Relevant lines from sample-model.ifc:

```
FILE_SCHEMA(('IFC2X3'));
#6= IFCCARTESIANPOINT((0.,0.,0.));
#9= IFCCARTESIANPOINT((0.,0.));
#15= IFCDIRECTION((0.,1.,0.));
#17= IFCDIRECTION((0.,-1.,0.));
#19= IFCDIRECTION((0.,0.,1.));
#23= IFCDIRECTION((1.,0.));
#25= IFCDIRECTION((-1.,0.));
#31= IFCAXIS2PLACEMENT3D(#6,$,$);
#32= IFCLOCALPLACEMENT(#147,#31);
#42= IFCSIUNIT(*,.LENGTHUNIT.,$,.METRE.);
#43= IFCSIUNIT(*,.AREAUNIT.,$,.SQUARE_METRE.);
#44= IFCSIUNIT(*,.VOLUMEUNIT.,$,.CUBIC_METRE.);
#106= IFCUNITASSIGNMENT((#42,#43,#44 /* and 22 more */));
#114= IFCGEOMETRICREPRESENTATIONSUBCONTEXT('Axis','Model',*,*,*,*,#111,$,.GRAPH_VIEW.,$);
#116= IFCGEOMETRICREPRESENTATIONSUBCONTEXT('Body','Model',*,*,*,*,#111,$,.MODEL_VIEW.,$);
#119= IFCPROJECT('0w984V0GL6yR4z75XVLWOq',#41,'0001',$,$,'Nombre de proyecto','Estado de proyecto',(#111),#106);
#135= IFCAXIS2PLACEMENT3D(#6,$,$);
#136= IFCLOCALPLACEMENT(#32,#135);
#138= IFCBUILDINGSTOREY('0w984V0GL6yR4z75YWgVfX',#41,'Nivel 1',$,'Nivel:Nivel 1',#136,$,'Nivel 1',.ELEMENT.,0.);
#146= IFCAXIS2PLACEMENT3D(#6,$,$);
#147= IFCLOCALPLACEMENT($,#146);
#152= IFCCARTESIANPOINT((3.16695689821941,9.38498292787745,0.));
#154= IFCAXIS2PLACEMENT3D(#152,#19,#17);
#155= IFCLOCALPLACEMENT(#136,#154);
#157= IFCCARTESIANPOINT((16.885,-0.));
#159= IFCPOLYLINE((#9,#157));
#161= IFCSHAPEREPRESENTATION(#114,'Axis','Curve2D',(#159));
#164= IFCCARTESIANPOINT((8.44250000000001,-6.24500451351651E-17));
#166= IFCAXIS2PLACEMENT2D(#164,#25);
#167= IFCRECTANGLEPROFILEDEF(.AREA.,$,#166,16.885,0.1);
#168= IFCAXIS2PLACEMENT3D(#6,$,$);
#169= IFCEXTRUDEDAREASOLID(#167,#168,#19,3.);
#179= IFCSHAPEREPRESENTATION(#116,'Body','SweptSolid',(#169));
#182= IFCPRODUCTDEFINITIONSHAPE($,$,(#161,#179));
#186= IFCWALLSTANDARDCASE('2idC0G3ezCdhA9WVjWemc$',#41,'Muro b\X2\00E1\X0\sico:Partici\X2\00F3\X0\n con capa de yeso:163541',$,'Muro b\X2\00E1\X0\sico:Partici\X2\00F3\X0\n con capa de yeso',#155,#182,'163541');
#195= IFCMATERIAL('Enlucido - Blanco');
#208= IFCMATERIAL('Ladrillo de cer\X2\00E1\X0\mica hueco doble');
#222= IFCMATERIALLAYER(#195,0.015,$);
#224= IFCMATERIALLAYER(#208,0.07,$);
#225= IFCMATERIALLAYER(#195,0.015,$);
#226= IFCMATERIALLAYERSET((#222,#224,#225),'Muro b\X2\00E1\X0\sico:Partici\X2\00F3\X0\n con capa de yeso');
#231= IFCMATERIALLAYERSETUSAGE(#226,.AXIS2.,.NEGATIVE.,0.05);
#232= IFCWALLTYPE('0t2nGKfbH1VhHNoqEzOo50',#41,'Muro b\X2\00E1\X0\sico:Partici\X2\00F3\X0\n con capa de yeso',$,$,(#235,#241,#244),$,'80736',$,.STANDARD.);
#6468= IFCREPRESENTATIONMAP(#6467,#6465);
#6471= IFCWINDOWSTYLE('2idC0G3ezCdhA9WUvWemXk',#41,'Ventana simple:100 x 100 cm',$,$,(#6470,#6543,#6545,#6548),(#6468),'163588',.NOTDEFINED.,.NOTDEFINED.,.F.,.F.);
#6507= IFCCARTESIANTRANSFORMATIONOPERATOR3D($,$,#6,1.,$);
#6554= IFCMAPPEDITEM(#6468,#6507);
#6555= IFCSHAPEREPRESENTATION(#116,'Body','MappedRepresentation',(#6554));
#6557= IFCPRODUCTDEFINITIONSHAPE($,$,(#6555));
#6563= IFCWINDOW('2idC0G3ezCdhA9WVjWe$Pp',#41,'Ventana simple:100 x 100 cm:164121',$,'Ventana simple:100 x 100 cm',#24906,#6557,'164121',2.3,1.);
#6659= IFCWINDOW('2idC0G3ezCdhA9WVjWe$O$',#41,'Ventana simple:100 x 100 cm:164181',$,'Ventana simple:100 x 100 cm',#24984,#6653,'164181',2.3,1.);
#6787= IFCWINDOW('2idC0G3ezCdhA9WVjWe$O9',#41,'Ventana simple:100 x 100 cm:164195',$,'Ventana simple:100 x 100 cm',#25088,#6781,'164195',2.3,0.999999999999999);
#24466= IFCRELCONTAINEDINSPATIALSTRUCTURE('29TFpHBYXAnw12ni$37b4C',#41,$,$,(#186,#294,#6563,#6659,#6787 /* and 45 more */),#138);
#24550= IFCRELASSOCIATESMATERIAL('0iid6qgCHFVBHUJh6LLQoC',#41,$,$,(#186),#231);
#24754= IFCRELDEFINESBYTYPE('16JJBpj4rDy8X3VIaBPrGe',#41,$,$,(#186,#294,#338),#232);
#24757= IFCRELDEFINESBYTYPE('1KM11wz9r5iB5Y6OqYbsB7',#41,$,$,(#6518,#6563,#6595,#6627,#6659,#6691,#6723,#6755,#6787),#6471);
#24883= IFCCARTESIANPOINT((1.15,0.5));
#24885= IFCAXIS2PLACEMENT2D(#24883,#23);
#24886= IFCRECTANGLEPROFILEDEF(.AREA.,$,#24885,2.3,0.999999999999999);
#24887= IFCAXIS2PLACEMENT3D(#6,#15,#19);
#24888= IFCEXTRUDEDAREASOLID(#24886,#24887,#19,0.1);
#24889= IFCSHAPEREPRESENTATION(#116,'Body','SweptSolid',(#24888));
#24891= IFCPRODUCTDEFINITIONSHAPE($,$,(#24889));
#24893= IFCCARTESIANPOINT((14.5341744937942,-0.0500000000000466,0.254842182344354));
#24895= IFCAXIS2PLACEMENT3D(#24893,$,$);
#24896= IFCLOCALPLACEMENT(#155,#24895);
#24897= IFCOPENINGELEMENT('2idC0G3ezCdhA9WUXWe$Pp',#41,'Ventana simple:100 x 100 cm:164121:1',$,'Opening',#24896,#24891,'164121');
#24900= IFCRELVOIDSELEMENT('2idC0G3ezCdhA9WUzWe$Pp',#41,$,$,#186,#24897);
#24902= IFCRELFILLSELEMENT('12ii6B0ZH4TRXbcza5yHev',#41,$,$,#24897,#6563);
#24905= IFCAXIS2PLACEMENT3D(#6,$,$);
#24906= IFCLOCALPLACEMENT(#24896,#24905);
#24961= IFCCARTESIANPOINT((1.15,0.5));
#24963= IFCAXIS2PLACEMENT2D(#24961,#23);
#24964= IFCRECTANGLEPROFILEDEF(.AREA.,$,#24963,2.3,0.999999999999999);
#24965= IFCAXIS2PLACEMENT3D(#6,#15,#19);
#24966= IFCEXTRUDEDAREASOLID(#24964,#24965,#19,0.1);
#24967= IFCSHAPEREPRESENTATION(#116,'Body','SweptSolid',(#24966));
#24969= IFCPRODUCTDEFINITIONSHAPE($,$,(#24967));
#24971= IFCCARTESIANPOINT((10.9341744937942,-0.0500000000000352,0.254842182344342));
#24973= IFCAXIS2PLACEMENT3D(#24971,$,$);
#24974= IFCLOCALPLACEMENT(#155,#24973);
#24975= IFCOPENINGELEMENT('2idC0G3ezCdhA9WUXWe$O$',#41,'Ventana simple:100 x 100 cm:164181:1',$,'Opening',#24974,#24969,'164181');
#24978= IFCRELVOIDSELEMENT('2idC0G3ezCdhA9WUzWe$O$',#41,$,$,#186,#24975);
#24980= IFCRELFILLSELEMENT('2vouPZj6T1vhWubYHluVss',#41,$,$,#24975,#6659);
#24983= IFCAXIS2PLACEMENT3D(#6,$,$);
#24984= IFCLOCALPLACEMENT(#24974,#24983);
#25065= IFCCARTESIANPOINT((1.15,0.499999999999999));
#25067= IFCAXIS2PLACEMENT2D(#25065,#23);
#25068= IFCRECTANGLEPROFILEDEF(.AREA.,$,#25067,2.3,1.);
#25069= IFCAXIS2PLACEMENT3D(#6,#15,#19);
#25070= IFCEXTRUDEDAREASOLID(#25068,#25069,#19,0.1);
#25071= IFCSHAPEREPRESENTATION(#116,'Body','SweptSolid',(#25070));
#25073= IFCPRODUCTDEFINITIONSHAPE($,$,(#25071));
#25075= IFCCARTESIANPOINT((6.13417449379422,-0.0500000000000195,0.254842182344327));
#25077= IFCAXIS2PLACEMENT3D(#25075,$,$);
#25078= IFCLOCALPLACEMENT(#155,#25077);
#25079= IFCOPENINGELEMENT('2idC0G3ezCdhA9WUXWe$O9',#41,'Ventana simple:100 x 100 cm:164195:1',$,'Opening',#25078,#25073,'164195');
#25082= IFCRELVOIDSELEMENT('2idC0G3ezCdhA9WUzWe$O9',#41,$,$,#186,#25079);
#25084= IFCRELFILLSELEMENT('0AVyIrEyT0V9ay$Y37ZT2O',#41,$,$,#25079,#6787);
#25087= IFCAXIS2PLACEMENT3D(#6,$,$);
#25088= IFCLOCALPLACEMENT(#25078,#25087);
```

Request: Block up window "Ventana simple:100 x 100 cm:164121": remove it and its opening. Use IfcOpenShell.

```python
import ifcopenshell
import ifcopenshell.api.feature
import ifcopenshell.api.root
import ifcopenshell.geom
import ifcopenshell.util.shape

model = ifcopenshell.open("sample-model.ifc")
settings = ifcopenshell.geom.settings()


def volume(element):
    """Net volume in cubic metres, openings subtracted."""
    shape = ifcopenshell.geom.create_shape(settings, element)
    return ifcopenshell.util.shape.get_volume(shape.geometry)


window = model.by_guid("2idC0G3ezCdhA9WVjWe$Pp")
opening = window.FillsVoids[0].RelatingOpeningElement
wall = opening.VoidsElements[0].RelatingBuildingElement
before = volume(wall)

ifcopenshell.api.root.remove_product(model, product=window)
ifcopenshell.api.feature.remove_feature(model, feature=opening)

after = volume(wall)

print(f"wall volume {before:.3f} -> {after:.3f} m3")

model.write("sample-model_updated.ifc")
```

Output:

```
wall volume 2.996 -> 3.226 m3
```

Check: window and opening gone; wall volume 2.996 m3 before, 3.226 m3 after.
